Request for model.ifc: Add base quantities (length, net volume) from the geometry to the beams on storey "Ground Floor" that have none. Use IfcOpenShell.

First a look at what the model holds.

```python
import ifcopenshell
import ifcopenshell.util.element
import ifcopenshell.util.unit

model = ifcopenshell.open("model.ifc")
print(model.schema)
for unit_type in ("LENGTHUNIT", "AREAUNIT", "VOLUMEUNIT"):
    print(unit_type, ifcopenshell.util.unit.calculate_unit_scale(model, unit_type))
storey = next(s for s in model.by_type("IfcBuildingStorey") if s.Name == "Ground Floor")
beams = [e for e in ifcopenshell.util.element.get_decomposition(storey) if e.is_a("IfcBeam")]
for e in sorted(beams, key=lambda e: e.id()):
    print(e.id(), e.is_a(), e.Name, list(ifcopenshell.util.element.get_psets(e, qtos_only=True)), sep=" | ")
```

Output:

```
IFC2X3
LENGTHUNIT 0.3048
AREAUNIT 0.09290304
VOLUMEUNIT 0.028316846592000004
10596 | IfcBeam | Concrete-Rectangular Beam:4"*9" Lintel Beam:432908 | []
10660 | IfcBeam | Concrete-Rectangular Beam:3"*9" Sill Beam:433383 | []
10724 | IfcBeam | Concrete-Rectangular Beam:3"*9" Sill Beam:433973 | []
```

```python
import ifcopenshell
import ifcopenshell.api.pset
import ifcopenshell.geom
import ifcopenshell.util.element
import ifcopenshell.util.shape
import ifcopenshell.util.unit

model = ifcopenshell.open("model.ifc")
unit_scale = ifcopenshell.util.unit.calculate_unit_scale(model)
volume_scale = ifcopenshell.util.unit.calculate_unit_scale(model, "VOLUMEUNIT")
settings = ifcopenshell.geom.settings()

storey = next(s for s in model.by_type("IfcBuildingStorey") if s.Name == "Ground Floor")
beams = [e for e in ifcopenshell.util.element.get_decomposition(storey) if e.is_a("IfcBeam")]

for e in sorted(beams, key=lambda e: e.id()):
    if ifcopenshell.util.element.get_psets(e, qtos_only=True, should_inherit=False):
        continue
    # Geometry comes back in metres, in the element's own axes.
    shape = ifcopenshell.geom.create_shape(settings, e)
    values = {
        "Length": ifcopenshell.util.shape.get_max_xyz(shape.geometry) / unit_scale,
        "NetVolume": ifcopenshell.util.shape.get_volume(shape.geometry) / volume_scale,
    }
    qto = ifcopenshell.api.pset.add_qto(model, product=e, name="BaseQuantities")
    ifcopenshell.api.pset.edit_qto(model, qto=qto, properties=values)
    print(e.id(), {k: round(v, 3) for k, v in values.items()})

model.write("model_edited.ifc")
```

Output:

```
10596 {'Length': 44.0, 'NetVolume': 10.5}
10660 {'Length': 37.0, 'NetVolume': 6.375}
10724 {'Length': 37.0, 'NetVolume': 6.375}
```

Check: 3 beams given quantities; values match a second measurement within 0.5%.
